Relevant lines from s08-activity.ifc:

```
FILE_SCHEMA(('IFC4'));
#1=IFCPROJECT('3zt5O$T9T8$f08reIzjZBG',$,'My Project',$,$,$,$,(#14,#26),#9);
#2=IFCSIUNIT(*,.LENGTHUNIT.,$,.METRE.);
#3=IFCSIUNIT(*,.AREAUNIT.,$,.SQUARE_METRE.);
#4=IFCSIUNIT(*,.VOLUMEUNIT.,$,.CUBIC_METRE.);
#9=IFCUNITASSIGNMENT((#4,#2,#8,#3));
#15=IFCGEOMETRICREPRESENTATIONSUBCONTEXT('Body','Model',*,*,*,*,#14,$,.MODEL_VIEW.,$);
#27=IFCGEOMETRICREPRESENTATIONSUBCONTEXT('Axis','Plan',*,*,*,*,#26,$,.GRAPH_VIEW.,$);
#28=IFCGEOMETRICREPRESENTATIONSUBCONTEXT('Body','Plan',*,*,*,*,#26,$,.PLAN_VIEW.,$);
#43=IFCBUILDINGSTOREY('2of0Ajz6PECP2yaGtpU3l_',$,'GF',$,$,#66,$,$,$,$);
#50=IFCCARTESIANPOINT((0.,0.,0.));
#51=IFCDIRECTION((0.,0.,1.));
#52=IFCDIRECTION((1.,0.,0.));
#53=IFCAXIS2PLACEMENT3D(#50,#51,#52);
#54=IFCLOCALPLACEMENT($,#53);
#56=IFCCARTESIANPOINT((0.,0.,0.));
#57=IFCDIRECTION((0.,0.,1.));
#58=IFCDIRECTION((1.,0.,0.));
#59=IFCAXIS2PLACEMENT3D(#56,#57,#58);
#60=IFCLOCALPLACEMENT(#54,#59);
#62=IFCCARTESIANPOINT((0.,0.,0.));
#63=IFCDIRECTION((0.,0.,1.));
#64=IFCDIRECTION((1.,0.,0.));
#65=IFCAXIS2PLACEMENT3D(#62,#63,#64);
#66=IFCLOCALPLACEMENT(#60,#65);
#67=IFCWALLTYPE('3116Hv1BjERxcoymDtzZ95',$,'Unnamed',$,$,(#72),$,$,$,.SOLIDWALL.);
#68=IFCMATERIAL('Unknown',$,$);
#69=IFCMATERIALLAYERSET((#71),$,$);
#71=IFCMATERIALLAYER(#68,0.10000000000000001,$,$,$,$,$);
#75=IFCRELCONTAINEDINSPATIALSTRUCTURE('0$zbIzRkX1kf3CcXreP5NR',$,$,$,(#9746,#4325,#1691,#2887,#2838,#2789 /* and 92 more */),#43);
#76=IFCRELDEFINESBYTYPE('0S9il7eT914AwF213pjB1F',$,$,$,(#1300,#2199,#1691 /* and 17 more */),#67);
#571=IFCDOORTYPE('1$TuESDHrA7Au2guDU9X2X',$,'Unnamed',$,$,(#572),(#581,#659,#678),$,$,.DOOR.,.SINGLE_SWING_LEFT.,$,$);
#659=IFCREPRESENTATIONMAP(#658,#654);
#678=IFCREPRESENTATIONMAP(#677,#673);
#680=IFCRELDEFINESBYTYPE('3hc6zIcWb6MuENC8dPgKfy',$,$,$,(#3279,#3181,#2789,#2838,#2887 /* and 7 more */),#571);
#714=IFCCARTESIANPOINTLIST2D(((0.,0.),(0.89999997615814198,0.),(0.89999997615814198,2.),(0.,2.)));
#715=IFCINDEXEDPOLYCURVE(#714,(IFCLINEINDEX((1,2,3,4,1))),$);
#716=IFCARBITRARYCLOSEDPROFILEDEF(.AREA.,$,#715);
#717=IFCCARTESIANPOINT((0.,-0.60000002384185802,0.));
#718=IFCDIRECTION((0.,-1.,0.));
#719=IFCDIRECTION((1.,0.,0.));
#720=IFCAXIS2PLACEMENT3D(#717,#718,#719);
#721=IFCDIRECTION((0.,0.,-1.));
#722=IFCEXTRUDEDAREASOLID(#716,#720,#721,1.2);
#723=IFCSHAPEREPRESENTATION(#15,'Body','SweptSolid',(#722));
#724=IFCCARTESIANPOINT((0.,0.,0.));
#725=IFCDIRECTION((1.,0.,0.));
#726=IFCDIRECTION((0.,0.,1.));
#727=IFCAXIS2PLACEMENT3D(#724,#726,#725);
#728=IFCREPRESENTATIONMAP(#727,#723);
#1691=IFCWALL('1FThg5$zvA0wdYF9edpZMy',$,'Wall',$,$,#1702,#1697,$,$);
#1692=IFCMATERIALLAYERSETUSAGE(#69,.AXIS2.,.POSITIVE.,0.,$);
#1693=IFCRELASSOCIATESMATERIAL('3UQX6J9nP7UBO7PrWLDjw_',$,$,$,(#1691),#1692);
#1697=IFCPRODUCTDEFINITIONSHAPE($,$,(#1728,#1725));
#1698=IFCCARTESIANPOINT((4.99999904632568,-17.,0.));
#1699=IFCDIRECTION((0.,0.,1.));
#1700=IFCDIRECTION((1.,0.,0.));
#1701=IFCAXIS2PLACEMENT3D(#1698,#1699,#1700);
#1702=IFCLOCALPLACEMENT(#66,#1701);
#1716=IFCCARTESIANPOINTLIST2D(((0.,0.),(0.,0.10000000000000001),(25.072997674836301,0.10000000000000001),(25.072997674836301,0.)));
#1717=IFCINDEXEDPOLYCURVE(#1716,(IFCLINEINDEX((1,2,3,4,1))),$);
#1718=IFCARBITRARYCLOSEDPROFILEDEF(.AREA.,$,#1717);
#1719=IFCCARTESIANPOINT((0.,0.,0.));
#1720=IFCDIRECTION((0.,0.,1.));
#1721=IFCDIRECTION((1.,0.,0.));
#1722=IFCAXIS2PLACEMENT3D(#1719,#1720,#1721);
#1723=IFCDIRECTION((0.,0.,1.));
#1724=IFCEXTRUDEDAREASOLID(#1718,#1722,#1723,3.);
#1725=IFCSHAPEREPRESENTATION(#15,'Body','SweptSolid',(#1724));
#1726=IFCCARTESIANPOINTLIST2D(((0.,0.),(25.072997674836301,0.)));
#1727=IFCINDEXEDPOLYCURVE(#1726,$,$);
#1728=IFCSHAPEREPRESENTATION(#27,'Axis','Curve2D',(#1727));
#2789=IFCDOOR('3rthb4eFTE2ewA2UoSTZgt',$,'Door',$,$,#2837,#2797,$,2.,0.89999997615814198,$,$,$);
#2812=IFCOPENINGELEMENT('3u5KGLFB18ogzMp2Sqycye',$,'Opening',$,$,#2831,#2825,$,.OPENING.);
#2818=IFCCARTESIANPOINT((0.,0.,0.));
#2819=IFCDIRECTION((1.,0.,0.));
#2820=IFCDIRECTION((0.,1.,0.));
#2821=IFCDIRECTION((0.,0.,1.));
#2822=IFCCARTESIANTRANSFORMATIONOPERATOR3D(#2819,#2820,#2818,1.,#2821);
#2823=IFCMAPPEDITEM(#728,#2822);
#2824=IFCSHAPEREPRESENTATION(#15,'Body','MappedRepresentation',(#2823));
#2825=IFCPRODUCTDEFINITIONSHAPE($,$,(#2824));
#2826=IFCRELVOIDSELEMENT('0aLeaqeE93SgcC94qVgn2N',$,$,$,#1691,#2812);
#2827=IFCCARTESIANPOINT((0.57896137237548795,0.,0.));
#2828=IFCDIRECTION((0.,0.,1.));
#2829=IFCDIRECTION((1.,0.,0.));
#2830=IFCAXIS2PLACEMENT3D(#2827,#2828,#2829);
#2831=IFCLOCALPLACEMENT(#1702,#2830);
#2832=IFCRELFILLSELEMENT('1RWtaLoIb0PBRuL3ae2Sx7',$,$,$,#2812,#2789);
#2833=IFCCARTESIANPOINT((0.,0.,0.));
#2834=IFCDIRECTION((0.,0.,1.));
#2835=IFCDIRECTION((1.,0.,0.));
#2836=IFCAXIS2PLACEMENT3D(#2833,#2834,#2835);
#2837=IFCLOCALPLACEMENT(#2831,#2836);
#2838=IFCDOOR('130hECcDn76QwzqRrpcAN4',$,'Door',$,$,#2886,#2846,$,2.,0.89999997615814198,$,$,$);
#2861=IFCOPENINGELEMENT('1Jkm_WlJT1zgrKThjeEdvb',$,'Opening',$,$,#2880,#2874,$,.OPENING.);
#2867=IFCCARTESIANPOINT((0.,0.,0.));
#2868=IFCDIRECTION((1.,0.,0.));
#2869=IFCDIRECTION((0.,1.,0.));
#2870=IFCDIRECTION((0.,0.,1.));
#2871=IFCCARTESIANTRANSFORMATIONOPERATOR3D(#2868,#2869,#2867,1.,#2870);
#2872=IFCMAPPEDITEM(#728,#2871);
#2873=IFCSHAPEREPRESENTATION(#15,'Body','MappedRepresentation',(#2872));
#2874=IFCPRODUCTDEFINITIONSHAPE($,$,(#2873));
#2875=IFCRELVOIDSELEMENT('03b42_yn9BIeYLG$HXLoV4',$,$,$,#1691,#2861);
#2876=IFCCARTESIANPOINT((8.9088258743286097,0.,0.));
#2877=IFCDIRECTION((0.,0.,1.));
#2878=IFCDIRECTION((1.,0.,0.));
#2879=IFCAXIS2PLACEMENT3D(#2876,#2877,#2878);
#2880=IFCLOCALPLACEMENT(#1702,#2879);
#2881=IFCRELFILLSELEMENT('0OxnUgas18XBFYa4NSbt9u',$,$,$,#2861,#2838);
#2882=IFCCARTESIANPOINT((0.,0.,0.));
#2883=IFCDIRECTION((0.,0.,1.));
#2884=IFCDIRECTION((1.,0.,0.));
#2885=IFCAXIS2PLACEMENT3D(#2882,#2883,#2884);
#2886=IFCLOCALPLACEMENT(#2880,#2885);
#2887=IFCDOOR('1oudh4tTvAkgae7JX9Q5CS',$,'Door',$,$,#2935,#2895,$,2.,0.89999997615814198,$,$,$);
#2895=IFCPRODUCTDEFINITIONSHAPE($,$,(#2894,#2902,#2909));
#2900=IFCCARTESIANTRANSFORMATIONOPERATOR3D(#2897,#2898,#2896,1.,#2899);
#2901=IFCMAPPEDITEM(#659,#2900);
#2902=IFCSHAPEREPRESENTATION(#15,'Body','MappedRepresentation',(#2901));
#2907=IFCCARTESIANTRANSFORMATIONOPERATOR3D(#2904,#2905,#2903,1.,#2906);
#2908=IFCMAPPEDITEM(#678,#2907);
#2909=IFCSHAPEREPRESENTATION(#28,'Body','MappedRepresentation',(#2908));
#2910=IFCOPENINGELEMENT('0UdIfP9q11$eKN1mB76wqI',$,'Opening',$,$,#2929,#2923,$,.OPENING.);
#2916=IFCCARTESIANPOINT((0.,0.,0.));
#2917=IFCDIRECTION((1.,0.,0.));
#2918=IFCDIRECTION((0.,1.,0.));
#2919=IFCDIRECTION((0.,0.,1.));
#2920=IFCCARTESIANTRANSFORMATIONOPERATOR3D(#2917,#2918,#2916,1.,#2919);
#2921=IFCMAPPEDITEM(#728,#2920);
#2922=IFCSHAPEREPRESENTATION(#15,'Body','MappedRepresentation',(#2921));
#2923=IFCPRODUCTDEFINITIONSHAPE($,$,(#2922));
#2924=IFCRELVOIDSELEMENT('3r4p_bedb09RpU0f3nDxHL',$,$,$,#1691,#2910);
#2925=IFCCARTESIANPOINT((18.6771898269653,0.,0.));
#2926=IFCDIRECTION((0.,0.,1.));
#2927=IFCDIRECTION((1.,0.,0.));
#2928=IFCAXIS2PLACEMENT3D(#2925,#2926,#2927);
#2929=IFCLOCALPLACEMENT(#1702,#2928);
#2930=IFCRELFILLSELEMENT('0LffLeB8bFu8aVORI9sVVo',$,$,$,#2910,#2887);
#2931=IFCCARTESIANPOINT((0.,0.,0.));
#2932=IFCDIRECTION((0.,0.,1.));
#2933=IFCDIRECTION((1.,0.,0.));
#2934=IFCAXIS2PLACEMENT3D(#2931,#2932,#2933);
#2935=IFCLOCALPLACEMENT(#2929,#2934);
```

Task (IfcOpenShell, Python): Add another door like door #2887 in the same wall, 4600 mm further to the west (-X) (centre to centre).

```python
import ifcopenshell
import ifcopenshell.api.feature
import ifcopenshell.api.geometry
import ifcopenshell.api.root
import ifcopenshell.geom
import ifcopenshell.util.element
import ifcopenshell.util.placement
import ifcopenshell.util.shape

model = ifcopenshell.open("s08-activity.ifc")
settings = ifcopenshell.geom.settings()


def volume(element):
    """Net volume in cubic metres, openings subtracted."""
    shape = ifcopenshell.geom.create_shape(settings, element)
    return ifcopenshell.util.shape.get_volume(shape.geometry)


door = model.by_id(2887)
opening = door.FillsVoids[0].RelatingOpeningElement
wall = opening.VoidsElements[0].RelatingBuildingElement
before = volume(wall)
shift = ifcopenshell.util.placement.get_local_placement(wall.ObjectPlacement)[:3, 0] * -4.6

# copy_class copies the void relationship, type, container and properties, but no geometry.
new_opening = ifcopenshell.api.root.copy_class(model, product=opening)
new_opening.Representation = ifcopenshell.util.element.copy_deep(
    model, opening.Representation, exclude=["IfcGeometricRepresentationContext", "IfcRepresentationMap"]
)
new_door = ifcopenshell.api.root.copy_class(model, product=door)
new_door.Representation = ifcopenshell.util.element.copy_deep(
    model, door.Representation, exclude=["IfcGeometricRepresentationContext", "IfcRepresentationMap"]
)
ifcopenshell.api.feature.add_filling(model, opening=new_opening, element=new_door)

for old, new in ((opening, new_opening), (door, new_door)):
    matrix = ifcopenshell.util.placement.get_local_placement(old.ObjectPlacement)
    matrix[:3, 3] += shift
    ifcopenshell.api.geometry.edit_object_placement(model, product=new, matrix=matrix, is_si=False)

after = volume(wall)

print(f"wall volume {before:.3f} -> {after:.3f} m3")

model.write("s08-activity_updated.ifc")
```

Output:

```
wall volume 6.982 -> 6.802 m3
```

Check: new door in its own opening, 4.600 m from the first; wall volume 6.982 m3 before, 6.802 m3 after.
